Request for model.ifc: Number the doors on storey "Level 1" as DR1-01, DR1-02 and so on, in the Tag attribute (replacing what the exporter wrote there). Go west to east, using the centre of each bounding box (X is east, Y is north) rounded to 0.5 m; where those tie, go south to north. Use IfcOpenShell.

First a look at what the model holds.

```python
import ifcopenshell
import ifcopenshell.util.element
import ifcopenshell.util.placement

model = ifcopenshell.open("model.ifc")
print(model.schema)
storey = next(s for s in model.by_type("IfcBuildingStorey") if s.Name == "Level 1")
doors = [e for e in ifcopenshell.util.element.get_decomposition(storey) if e.is_a("IfcDoor")]
for e in sorted(doors, key=lambda e: e.id()):
    origin = ifcopenshell.util.placement.get_local_placement(e.ObjectPlacement)[:3, 3]
    print(e.id(), e.Tag, e.Name, origin.round(2) + 0.0, sep=" | ")
```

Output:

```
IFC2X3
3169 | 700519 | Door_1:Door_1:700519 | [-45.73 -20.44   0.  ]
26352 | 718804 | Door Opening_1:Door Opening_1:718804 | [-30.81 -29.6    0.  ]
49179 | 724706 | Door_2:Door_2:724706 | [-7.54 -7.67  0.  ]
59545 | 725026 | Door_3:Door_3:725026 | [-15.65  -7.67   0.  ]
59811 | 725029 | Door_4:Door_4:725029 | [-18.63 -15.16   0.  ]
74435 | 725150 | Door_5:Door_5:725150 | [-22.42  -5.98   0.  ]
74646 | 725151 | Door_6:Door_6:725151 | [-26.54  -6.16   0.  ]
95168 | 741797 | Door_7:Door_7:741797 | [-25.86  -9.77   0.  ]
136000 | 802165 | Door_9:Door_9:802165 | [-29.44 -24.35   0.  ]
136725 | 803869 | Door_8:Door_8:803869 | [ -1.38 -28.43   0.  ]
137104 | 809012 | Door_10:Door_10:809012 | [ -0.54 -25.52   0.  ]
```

```python
import ifcopenshell
import ifcopenshell.geom
import ifcopenshell.util.element
import ifcopenshell.util.shape

model = ifcopenshell.open("model.ifc")
settings = ifcopenshell.geom.settings()
settings.set("use-world-coords", True)


def centre(element):
    shape = ifcopenshell.geom.create_shape(settings, element)
    return ifcopenshell.util.shape.get_bbox_centroid(shape.geometry)


storey = next(s for s in model.by_type("IfcBuildingStorey") if s.Name == "Level 1")
doors = [e for e in ifcopenshell.util.element.get_decomposition(storey) if e.is_a("IfcDoor")]

# Insertion points can sit at a corner or the storey origin, so sort by the geometry (in metres).
centres = {e: centre(e) for e in doors}
doors.sort(key=lambda e: (round(centres[e][0] / 0.5), centres[e][1]))

for i, e in enumerate(doors, start=1):
    number = f"DR1-{i:02d}"
    e.Tag = number
    print(e.id(), number)

model.write("model_updated.ifc")
```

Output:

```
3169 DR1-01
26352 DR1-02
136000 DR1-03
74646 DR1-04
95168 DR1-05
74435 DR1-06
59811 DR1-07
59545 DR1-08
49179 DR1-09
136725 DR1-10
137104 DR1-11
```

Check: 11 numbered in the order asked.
